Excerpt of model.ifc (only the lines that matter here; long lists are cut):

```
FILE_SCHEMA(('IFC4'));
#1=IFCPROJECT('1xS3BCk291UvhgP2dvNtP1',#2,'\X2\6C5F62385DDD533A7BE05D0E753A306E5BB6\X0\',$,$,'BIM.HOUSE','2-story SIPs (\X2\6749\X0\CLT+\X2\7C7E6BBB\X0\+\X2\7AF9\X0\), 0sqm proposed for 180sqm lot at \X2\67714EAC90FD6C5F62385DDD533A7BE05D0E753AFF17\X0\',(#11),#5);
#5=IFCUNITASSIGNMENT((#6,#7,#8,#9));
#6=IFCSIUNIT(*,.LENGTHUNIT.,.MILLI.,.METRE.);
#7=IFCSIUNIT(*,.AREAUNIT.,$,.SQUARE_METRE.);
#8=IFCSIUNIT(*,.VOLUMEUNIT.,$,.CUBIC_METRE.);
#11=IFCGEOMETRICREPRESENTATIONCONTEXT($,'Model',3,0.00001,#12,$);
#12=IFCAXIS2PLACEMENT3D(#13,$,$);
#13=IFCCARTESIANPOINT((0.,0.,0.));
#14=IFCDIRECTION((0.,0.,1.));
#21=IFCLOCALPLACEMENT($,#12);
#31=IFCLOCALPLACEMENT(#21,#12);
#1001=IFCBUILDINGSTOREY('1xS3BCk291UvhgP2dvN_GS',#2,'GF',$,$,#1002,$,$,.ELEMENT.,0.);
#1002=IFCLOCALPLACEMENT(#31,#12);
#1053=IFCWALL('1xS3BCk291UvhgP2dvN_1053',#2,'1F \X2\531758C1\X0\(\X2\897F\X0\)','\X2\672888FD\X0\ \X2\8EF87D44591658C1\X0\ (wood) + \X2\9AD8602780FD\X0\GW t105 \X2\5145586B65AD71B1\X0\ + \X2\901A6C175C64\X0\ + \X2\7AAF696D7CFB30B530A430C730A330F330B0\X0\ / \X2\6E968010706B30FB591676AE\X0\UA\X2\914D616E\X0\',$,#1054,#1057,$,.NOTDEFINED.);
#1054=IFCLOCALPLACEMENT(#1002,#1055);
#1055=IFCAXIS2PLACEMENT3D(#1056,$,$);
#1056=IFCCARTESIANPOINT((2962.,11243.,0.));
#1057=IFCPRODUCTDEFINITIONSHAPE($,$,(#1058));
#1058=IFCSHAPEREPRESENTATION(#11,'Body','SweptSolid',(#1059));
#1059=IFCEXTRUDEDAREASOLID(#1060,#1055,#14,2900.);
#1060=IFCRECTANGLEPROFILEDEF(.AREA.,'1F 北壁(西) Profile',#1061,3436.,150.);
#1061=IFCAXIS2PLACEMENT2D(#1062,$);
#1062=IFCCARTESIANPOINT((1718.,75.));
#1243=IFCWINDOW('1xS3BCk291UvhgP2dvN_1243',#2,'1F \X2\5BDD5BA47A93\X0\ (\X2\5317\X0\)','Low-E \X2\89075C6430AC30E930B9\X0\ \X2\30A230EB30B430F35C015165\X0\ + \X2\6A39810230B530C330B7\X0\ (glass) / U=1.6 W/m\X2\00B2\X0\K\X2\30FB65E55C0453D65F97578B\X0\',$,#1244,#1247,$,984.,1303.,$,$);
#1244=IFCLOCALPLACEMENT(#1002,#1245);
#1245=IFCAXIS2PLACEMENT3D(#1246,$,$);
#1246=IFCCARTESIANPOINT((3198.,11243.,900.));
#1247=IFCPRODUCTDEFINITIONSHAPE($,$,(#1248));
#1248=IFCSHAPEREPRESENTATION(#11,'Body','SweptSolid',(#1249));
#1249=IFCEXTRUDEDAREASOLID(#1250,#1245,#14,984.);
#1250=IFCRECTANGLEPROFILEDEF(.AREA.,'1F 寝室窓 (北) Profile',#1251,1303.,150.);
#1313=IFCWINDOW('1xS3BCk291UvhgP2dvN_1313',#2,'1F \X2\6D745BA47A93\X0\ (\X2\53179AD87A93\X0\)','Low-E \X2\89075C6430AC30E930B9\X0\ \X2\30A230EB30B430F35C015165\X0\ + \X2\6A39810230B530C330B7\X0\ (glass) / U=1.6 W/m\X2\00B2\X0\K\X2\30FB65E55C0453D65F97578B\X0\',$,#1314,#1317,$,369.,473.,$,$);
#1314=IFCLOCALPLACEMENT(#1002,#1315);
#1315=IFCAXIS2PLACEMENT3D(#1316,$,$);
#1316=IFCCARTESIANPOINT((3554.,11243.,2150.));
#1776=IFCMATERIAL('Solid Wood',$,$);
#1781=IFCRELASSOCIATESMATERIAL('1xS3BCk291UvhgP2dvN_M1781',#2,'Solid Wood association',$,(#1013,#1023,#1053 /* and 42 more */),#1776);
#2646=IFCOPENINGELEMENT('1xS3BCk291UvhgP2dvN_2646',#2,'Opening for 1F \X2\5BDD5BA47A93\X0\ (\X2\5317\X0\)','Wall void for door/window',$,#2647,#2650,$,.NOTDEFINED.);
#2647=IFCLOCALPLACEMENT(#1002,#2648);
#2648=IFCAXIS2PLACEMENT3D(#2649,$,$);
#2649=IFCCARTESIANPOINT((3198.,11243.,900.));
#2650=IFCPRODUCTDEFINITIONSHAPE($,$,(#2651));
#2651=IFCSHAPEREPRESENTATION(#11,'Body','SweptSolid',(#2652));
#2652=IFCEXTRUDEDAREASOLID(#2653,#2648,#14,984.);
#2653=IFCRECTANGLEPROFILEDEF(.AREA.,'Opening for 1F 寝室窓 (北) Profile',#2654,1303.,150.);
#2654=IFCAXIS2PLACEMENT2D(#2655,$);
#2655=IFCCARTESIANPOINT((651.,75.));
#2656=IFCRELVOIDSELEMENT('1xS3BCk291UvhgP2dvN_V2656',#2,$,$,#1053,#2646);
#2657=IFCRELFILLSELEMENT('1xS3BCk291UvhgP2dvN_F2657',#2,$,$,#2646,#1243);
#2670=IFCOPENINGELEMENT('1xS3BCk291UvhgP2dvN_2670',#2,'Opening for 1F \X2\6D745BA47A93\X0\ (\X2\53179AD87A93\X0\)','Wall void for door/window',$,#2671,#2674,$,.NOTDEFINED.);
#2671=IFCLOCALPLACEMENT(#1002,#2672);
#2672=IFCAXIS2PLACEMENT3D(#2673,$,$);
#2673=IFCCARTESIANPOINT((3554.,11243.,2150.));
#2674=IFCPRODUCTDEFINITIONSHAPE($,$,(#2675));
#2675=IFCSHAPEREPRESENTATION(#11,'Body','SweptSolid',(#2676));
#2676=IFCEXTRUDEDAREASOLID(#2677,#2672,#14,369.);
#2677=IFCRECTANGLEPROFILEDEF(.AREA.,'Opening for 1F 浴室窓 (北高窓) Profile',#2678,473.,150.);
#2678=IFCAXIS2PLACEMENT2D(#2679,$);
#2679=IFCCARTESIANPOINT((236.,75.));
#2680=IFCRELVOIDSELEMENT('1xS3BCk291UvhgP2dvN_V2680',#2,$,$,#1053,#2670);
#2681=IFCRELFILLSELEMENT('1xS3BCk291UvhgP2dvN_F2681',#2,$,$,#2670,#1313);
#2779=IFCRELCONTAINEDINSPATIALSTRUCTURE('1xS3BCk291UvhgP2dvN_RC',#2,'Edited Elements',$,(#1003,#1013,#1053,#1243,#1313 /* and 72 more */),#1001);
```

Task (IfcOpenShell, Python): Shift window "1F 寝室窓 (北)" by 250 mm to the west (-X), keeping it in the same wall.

```python
import ifcopenshell
import ifcopenshell.api.geometry
import ifcopenshell.util.placement
import ifcopenshell.util.unit

model = ifcopenshell.open("model.ifc")
unit_scale = ifcopenshell.util.unit.calculate_unit_scale(model)

window = model.by_guid("1xS3BCk291UvhgP2dvN_1243")
opening = window.FillsVoids[0].RelatingOpeningElement
wall = opening.VoidsElements[0].RelatingBuildingElement

wall_matrix = ifcopenshell.util.placement.get_local_placement(wall.ObjectPlacement)
shift = wall_matrix[:3, 0] * -0.25 / unit_scale
before = ifcopenshell.util.placement.get_local_placement(window.ObjectPlacement)[:3, 3].copy()

# The window is not placed relative to its opening, so move both.
for product in (opening, window):
    matrix = ifcopenshell.util.placement.get_local_placement(product.ObjectPlacement)
    matrix[:3, 3] += shift
    ifcopenshell.api.geometry.edit_object_placement(model, product=product, matrix=matrix, is_si=False)

after = ifcopenshell.util.placement.get_local_placement(window.ObjectPlacement)[:3, 3]
print("window moved by", (after - before).round(3) + 0.0)

model.write("model_rev.ifc")
```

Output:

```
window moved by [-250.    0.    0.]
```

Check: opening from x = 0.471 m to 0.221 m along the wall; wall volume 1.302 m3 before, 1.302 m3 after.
